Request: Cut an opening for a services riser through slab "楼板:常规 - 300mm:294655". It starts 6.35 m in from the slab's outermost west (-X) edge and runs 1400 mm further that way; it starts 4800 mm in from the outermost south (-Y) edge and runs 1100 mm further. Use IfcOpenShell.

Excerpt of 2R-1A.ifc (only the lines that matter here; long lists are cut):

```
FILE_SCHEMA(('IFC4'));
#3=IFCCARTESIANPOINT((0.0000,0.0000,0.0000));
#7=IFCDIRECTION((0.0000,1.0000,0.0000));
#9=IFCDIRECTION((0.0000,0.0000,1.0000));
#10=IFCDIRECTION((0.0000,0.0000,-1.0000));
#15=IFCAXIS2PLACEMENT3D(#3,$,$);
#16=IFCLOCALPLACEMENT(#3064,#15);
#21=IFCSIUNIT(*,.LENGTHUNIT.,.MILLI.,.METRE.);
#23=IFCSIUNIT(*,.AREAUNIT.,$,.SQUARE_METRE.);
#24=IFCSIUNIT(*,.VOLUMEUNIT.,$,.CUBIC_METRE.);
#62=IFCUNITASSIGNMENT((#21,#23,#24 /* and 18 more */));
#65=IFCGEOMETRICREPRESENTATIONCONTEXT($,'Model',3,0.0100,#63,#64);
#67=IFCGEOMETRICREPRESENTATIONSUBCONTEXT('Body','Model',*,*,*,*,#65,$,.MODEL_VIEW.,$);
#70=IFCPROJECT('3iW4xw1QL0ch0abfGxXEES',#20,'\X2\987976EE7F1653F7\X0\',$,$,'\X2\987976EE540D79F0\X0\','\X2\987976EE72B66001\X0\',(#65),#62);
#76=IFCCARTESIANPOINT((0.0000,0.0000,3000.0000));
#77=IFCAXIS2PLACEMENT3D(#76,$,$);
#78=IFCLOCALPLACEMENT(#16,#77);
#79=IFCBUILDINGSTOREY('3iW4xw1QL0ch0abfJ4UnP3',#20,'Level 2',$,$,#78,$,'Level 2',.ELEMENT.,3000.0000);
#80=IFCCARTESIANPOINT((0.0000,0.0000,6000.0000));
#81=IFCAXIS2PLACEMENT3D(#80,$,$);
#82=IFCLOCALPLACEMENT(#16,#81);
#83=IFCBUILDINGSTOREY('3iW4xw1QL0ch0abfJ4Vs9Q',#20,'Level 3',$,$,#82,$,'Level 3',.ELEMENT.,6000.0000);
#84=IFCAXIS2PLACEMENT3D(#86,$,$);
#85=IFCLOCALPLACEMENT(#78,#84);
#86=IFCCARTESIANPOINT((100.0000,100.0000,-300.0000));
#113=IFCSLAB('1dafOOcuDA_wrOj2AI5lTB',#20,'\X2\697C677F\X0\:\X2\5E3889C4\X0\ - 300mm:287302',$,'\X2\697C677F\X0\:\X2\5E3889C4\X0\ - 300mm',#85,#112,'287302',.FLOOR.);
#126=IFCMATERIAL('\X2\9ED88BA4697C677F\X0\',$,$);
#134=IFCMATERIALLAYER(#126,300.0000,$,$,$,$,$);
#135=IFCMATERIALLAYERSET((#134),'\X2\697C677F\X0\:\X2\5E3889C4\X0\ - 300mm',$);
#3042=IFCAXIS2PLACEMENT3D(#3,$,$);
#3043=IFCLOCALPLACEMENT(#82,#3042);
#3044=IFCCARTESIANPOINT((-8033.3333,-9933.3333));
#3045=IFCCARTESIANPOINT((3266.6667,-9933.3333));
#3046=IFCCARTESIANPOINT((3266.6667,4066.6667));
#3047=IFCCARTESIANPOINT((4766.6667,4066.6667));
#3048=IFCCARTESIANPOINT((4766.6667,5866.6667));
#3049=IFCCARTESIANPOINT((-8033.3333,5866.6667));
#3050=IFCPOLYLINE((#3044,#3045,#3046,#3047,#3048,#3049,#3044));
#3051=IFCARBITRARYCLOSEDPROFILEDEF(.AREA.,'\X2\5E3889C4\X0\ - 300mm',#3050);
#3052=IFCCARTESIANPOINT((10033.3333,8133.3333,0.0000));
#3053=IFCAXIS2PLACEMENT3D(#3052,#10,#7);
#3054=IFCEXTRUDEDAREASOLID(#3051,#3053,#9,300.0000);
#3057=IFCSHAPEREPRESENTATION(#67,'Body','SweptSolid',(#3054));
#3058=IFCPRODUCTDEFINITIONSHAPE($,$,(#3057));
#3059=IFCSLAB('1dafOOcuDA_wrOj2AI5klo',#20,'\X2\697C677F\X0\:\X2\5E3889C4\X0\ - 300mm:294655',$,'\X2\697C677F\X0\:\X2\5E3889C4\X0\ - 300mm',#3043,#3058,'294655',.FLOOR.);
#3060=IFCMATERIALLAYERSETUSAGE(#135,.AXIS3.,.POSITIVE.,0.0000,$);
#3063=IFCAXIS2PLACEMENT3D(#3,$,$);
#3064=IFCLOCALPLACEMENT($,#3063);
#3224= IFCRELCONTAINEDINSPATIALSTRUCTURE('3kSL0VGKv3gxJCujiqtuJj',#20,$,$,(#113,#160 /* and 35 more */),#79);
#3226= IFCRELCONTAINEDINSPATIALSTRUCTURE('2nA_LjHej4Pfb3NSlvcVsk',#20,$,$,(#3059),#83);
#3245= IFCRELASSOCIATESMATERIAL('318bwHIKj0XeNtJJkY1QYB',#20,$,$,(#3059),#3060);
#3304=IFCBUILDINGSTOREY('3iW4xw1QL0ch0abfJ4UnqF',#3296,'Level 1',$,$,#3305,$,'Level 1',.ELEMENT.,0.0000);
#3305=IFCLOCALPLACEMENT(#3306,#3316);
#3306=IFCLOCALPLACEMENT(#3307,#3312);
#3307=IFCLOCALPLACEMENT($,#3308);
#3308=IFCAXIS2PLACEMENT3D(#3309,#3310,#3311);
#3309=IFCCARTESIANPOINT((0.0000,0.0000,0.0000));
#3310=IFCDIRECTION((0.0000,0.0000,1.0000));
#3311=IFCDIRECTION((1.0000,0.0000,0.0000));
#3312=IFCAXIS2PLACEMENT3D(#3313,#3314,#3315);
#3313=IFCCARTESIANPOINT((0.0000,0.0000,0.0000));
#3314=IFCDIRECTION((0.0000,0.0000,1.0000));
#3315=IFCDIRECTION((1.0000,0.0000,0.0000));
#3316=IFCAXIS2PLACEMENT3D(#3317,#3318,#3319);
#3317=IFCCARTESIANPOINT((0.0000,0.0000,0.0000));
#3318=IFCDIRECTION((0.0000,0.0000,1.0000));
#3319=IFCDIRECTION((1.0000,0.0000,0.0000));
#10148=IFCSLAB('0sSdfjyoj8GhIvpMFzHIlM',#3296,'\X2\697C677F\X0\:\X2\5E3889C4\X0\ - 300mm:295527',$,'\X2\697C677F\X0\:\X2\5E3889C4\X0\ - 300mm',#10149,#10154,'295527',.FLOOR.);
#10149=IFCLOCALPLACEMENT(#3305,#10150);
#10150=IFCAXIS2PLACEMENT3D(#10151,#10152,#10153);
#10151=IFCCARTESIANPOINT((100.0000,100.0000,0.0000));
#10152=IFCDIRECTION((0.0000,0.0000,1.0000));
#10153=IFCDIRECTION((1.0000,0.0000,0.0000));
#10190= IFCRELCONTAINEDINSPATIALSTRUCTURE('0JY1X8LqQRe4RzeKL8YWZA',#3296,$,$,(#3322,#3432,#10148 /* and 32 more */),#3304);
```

```python
import numpy as np
import ifcopenshell
import ifcopenshell.api.feature
import ifcopenshell.api.geometry
import ifcopenshell.api.root
import ifcopenshell.geom
import ifcopenshell.util.placement
import ifcopenshell.util.representation
import ifcopenshell.util.shape
import ifcopenshell.util.unit

model = ifcopenshell.open("2R-1A.ifc")
unit_scale = ifcopenshell.util.unit.calculate_unit_scale(model)
settings = ifcopenshell.geom.settings()


def volume(element):
    """Net volume in cubic metres, openings subtracted."""
    shape = ifcopenshell.geom.create_shape(settings, element)
    return ifcopenshell.util.shape.get_volume(shape.geometry)


slab = model.by_guid("1dafOOcuDA_wrOj2AI5klo")
before = volume(slab)

# Extent in the slab's own axes, in metres. The edges named are its -X and -Y sides.
slab_shape = ifcopenshell.geom.create_shape(settings, slab)
vertices = ifcopenshell.util.shape.get_vertices(slab_shape.geometry)
x_min, y_min, bottom = vertices.min(axis=0)
top = vertices[:, 2].max()

opening = ifcopenshell.api.root.create_entity(model, ifc_class="IfcOpeningElement", name="Services riser opening", predefined_type="OPENING")
context = ifcopenshell.util.representation.get_context(model, "Model", "Body", "MODEL_VIEW")
width, depth = 1.4, 1.1
outline = [(0.0, 0.0), (width, 0.0), (width, depth), (0.0, depth), (0.0, 0.0)]
# Overshoot both faces by 50 mm so the cut is clean.
shape = ifcopenshell.api.geometry.add_slab_representation(
    model, context=context, depth=top - bottom + 0.1, polyline=outline
)
ifcopenshell.api.geometry.assign_representation(model, product=opening, representation=shape)

matrix = ifcopenshell.util.placement.get_local_placement(slab.ObjectPlacement)
matrix[:, 3] = matrix @ np.append(np.array([x_min + 6.35, y_min + 4.8, bottom - 0.05]) / unit_scale, 1.0)
ifcopenshell.api.geometry.edit_object_placement(model, product=opening, matrix=matrix, is_si=False)
ifcopenshell.api.feature.add_feature(model, feature=opening, element=slab)

after = volume(slab)

print(f"slab volume {before:.3f} -> {after:.3f} m3")

model.write("2R-1A-out.ifc")
```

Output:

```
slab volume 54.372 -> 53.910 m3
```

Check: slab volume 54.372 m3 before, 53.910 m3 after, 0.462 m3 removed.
